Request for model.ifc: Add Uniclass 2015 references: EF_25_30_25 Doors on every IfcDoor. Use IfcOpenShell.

First a look at what the model holds.

```python
import ifcopenshell

model = ifcopenshell.open("model.ifc")
print(model.schema)
print("classifications:", [c.Name for c in model.by_type("IfcClassification")])
for ifc_class in ("IfcDoor", "IfcRoof", "IfcStair", "IfcWall", "IfcWindow"):
    print(ifc_class, len(model.by_type(ifc_class)))
```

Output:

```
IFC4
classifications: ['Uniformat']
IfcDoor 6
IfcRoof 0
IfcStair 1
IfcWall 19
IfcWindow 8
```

```python
import ifcopenshell
import ifcopenshell.api.classification

model = ifcopenshell.open("model.ifc")

system = ifcopenshell.api.classification.add_classification(model, classification="Uniclass 2015")

codes = {
    "IfcDoor": ("EF_25_30_25", "Doors"),
}
for ifc_class, (code, name) in codes.items():
    products = model.by_type(ifc_class)
    ifcopenshell.api.classification.add_reference(
        model, products=products, classification=system, identification=code, name=name
    )
    print(code, len(products))

model.write("model_rev.ifc")
```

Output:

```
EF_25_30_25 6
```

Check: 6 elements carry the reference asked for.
